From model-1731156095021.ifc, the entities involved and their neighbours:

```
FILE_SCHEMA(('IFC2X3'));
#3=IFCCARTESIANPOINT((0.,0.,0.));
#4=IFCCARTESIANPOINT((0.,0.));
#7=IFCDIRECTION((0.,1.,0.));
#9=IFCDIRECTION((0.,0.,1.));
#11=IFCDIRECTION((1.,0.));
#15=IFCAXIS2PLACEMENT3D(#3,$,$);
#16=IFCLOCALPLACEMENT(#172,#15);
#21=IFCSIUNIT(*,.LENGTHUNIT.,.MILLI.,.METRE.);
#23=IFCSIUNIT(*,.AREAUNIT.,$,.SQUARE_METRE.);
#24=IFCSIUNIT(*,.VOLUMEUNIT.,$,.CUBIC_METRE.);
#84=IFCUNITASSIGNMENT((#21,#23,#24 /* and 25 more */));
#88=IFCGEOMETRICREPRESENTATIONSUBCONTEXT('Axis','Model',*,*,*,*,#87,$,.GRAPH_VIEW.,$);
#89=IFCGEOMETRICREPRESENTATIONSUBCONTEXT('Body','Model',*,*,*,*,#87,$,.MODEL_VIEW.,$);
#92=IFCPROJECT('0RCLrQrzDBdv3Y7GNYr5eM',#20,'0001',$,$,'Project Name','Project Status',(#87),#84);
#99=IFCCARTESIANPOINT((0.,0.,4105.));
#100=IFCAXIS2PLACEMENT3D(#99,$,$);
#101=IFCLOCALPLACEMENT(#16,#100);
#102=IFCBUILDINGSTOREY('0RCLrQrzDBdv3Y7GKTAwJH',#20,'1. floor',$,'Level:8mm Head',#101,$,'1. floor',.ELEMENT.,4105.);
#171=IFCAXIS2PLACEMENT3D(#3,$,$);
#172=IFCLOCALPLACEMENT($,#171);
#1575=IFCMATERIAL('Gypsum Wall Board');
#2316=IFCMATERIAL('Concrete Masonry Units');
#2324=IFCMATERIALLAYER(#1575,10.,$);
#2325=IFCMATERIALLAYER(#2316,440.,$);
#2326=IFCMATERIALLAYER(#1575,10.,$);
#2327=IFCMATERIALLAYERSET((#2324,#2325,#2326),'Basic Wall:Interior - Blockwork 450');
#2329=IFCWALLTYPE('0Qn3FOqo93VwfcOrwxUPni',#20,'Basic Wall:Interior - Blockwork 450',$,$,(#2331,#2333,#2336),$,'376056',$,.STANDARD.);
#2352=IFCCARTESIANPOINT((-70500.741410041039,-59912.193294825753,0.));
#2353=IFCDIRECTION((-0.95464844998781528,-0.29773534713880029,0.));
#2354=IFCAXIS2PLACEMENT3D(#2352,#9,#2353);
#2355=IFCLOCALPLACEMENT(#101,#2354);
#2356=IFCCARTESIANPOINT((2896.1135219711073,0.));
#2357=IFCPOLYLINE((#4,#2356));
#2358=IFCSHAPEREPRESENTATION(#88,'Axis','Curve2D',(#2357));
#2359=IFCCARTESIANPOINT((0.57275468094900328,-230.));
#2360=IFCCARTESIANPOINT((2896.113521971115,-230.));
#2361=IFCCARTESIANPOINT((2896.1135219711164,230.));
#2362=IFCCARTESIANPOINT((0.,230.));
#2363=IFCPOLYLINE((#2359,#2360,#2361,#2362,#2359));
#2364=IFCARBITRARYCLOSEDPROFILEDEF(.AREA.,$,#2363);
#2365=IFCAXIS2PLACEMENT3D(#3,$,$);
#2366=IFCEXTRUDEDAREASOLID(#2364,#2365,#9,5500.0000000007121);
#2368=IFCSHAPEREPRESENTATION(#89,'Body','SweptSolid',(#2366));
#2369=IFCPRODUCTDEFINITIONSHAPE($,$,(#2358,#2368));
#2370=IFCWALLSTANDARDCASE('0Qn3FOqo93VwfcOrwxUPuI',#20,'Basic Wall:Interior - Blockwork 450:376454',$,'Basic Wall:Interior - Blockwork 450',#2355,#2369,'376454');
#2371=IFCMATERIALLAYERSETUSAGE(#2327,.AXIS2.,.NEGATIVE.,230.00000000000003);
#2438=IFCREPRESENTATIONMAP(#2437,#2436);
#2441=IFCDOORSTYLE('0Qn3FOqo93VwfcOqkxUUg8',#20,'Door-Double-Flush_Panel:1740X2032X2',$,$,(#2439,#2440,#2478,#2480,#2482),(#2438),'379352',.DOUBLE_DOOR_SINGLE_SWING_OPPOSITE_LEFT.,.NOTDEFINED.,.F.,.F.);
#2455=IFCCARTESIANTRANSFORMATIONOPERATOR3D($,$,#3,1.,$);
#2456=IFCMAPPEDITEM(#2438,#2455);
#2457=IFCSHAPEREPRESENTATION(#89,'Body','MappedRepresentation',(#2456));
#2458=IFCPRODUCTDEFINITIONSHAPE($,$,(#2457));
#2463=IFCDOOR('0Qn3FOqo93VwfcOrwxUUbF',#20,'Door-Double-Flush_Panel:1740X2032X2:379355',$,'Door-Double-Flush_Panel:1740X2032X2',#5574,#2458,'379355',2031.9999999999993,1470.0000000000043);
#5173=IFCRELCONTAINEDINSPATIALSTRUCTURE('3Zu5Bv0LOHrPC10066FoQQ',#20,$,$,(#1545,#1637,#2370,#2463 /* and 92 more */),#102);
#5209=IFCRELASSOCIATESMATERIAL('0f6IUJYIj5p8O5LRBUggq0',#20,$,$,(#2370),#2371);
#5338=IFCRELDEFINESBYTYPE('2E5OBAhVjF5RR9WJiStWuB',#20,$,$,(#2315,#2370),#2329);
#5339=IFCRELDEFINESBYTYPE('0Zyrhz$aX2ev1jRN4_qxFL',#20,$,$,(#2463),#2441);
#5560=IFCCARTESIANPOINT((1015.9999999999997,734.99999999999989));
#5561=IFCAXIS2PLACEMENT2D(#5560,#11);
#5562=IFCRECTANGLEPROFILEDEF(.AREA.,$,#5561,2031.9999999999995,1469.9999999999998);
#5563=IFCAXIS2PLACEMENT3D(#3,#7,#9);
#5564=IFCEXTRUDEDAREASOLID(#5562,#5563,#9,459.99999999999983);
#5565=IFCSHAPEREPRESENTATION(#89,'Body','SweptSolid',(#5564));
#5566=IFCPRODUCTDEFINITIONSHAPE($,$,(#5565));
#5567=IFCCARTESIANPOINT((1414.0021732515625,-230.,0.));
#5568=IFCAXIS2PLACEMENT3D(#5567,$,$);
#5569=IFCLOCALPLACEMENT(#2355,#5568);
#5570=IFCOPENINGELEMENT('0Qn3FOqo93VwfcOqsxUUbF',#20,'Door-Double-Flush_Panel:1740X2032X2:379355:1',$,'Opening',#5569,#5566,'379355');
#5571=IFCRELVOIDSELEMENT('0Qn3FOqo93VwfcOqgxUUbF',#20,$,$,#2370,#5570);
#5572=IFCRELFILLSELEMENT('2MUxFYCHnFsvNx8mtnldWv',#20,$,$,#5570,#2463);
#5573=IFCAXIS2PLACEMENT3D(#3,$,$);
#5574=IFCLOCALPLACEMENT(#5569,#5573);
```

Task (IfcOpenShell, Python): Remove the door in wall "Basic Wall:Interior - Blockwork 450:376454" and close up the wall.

```python
import ifcopenshell
import ifcopenshell.api.feature
import ifcopenshell.api.root
import ifcopenshell.geom
import ifcopenshell.util.shape

model = ifcopenshell.open("model-1731156095021.ifc")
settings = ifcopenshell.geom.settings()


def volume(element):
    """Net volume in cubic metres, openings subtracted."""
    shape = ifcopenshell.geom.create_shape(settings, element)
    return ifcopenshell.util.shape.get_volume(shape.geometry)


door = model.by_guid("0Qn3FOqo93VwfcOrwxUUbF")
opening = door.FillsVoids[0].RelatingOpeningElement
wall = opening.VoidsElements[0].RelatingBuildingElement
before = volume(wall)

ifcopenshell.api.root.remove_product(model, product=door)
ifcopenshell.api.feature.remove_feature(model, feature=opening)

after = volume(wall)

print(f"wall volume {before:.3f} -> {after:.3f} m3")

model.write("model-1731156095021_v2.ifc")
```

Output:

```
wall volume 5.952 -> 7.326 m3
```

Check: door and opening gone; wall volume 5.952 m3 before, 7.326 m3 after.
